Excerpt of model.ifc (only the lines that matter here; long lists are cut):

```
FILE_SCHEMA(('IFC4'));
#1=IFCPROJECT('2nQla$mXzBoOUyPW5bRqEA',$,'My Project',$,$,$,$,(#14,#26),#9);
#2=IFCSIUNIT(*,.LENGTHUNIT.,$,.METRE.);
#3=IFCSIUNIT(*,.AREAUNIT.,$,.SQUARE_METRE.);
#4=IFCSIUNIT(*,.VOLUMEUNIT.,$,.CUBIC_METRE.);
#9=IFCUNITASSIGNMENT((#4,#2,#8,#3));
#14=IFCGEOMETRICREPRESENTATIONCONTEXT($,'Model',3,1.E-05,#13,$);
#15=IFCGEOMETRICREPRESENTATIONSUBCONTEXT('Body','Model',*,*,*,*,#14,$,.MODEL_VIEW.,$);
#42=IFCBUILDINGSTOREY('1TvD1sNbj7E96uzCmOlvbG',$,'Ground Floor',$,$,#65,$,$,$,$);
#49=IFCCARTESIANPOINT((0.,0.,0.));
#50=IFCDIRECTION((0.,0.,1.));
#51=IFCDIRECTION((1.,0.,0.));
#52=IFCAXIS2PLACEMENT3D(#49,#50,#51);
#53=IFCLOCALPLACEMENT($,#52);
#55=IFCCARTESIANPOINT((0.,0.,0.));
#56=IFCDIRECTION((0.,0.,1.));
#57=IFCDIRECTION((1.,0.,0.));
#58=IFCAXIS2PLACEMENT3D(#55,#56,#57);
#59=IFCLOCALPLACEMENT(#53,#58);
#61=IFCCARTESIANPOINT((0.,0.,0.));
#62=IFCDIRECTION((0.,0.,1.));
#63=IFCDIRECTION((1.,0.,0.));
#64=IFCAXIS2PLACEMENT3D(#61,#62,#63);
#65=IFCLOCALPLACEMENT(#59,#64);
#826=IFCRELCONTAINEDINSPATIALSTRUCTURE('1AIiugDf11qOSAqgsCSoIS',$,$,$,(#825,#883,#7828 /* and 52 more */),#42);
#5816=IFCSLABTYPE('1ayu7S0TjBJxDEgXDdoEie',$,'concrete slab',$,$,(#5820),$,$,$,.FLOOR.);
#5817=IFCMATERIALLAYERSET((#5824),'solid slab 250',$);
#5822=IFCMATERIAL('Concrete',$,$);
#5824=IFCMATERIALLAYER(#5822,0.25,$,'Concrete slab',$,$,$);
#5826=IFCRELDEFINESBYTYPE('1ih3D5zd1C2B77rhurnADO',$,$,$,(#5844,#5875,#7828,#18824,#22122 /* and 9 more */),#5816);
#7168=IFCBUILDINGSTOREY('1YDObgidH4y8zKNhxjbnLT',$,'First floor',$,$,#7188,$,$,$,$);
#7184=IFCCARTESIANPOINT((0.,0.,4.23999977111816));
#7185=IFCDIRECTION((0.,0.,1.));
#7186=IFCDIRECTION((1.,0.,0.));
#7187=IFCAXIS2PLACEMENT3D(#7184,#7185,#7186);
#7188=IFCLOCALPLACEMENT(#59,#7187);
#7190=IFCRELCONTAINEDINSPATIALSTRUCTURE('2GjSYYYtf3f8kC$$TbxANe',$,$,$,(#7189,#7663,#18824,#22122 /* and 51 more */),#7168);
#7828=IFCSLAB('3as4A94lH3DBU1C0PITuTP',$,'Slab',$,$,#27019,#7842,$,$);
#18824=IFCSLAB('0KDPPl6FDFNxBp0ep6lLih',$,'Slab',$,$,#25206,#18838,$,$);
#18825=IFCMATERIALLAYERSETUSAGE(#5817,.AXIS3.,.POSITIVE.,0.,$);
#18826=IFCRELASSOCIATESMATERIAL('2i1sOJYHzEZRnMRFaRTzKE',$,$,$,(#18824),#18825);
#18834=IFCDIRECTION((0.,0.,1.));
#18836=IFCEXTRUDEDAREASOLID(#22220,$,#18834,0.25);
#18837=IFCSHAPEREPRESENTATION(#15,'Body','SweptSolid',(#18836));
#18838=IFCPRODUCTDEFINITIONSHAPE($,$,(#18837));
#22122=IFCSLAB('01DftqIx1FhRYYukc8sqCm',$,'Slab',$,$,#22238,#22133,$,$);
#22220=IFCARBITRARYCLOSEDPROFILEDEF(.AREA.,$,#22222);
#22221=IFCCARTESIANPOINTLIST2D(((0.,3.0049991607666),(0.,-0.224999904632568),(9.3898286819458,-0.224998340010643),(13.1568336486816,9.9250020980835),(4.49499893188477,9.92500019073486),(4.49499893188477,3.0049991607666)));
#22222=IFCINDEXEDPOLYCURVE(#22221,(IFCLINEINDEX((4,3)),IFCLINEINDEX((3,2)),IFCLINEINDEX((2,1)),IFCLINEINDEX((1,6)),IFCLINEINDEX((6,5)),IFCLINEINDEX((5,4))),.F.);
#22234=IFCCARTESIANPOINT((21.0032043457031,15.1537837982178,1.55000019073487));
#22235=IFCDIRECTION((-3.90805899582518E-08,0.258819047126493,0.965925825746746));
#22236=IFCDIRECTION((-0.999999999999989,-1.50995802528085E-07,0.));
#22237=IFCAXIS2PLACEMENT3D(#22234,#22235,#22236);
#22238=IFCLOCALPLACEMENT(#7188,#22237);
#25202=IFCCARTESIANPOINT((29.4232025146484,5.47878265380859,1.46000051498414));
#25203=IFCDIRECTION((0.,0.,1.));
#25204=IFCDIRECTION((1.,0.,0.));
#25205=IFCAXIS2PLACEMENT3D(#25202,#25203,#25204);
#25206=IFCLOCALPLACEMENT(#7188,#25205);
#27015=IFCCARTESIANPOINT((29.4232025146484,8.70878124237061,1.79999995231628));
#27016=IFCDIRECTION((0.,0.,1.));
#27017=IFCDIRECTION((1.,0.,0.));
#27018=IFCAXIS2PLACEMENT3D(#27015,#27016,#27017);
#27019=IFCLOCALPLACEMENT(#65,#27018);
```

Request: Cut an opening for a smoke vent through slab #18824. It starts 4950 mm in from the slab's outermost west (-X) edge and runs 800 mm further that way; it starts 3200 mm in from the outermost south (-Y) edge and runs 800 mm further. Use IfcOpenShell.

```python
import numpy as np
import ifcopenshell
import ifcopenshell.api.feature
import ifcopenshell.api.geometry
import ifcopenshell.api.root
import ifcopenshell.geom
import ifcopenshell.util.placement
import ifcopenshell.util.representation
import ifcopenshell.util.shape
import ifcopenshell.util.unit

model = ifcopenshell.open("model.ifc")
unit_scale = ifcopenshell.util.unit.calculate_unit_scale(model)
settings = ifcopenshell.geom.settings()


def volume(element):
    """Net volume in cubic metres, openings subtracted."""
    shape = ifcopenshell.geom.create_shape(settings, element)
    return ifcopenshell.util.shape.get_volume(shape.geometry)


slab = model.by_id(18824)
before = volume(slab)

# Extent in the slab's own axes, in metres. The edges named are its -X and -Y sides.
slab_shape = ifcopenshell.geom.create_shape(settings, slab)
vertices = ifcopenshell.util.shape.get_vertices(slab_shape.geometry)
x_min, y_min, bottom = vertices.min(axis=0)
top = vertices[:, 2].max()

opening = ifcopenshell.api.root.create_entity(model, ifc_class="IfcOpeningElement", name="Smoke vent opening", predefined_type="OPENING")
context = ifcopenshell.util.representation.get_context(model, "Model", "Body", "MODEL_VIEW")
width, depth = 0.8, 0.8
outline = [(0.0, 0.0), (width, 0.0), (width, depth), (0.0, depth), (0.0, 0.0)]
# Overshoot both faces by 50 mm so the cut is clean.
shape = ifcopenshell.api.geometry.add_slab_representation(
    model, context=context, depth=top - bottom + 0.1, polyline=outline
)
ifcopenshell.api.geometry.assign_representation(model, product=opening, representation=shape)

matrix = ifcopenshell.util.placement.get_local_placement(slab.ObjectPlacement)
matrix[:, 3] = matrix @ np.append(np.array([x_min + 4.95, y_min + 3.2, bottom - 0.05]) / unit_scale, 1.0)
ifcopenshell.api.geometry.edit_object_placement(model, product=opening, matrix=matrix, is_si=False)
ifcopenshell.api.feature.add_feature(model, feature=opening, element=slab)

after = volume(slab)

print(f"slab volume {before:.3f} -> {after:.3f} m3")

model.write("model-out.ifc")
```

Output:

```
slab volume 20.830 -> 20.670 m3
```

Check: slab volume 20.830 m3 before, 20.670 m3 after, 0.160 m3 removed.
